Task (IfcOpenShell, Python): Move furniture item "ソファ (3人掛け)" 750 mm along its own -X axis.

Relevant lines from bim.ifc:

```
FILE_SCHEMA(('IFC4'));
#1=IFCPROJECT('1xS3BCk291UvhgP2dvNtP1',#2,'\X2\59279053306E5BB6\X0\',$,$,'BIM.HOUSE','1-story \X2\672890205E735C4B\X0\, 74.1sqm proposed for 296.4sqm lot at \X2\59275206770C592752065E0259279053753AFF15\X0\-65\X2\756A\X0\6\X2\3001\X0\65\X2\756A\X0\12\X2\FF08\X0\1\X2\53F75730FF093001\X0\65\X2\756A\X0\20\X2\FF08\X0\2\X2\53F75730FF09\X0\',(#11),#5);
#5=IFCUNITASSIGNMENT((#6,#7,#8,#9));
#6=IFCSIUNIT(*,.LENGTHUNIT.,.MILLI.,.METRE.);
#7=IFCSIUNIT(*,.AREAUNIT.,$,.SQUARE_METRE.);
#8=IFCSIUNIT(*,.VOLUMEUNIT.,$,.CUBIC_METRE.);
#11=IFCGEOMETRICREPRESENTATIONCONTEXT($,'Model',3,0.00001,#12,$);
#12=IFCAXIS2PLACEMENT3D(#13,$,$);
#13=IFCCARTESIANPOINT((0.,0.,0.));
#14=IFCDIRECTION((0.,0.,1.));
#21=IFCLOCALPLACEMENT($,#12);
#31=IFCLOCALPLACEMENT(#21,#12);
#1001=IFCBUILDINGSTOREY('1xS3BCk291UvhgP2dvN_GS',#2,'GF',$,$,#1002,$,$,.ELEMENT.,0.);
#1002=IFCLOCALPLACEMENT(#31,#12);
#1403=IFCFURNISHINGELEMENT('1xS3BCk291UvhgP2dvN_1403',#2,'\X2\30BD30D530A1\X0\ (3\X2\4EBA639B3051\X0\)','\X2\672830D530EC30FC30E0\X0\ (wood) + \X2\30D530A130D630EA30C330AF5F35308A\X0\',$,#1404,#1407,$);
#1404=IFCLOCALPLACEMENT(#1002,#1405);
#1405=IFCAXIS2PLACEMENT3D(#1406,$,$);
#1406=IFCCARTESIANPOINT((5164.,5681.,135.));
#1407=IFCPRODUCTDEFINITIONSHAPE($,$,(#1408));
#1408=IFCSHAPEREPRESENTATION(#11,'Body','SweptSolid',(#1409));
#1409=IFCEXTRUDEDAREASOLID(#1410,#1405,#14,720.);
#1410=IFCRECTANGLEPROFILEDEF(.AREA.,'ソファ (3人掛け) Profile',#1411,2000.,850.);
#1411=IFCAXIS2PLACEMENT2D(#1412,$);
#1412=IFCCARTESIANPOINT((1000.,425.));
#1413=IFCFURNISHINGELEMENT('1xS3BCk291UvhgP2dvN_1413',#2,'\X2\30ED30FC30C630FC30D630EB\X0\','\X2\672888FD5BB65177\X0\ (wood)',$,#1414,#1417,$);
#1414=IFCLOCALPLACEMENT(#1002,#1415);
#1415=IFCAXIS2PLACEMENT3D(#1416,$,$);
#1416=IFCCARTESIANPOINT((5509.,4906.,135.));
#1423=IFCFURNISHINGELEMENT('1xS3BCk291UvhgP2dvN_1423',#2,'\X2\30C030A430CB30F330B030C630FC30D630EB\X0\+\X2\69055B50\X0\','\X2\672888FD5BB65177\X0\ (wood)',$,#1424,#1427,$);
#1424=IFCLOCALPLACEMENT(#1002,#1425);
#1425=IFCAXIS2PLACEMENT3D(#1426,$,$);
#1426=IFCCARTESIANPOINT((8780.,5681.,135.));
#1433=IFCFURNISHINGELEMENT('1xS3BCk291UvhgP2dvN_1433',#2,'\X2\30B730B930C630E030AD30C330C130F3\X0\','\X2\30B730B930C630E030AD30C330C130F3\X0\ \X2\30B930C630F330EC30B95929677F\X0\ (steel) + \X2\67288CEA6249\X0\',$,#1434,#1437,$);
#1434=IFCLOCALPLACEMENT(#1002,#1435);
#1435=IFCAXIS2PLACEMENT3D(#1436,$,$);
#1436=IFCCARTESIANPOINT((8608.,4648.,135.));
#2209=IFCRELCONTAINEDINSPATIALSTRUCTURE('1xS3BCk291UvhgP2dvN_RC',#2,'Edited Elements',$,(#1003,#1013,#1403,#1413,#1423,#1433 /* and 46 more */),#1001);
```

```python
import ifcopenshell
import ifcopenshell.api.geometry
import ifcopenshell.util.placement
import ifcopenshell.util.unit

model = ifcopenshell.open("bim.ifc")
unit_scale = ifcopenshell.util.unit.calculate_unit_scale(model)

item = model.by_id(1403)
matrix = ifcopenshell.util.placement.get_local_placement(item.ObjectPlacement)
matrix[:3, 3] -= matrix[:3, 0] * 0.75 / unit_scale
ifcopenshell.api.geometry.edit_object_placement(model, product=item, matrix=matrix, is_si=False)

print(ifcopenshell.util.placement.get_local_placement(item.ObjectPlacement).round(3) + 0.0)

model.write("bim_updated.ifc")
```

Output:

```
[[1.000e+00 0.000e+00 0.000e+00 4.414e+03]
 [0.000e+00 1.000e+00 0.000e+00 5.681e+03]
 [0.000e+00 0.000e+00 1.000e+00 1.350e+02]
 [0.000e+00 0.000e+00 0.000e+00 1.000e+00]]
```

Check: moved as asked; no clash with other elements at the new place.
